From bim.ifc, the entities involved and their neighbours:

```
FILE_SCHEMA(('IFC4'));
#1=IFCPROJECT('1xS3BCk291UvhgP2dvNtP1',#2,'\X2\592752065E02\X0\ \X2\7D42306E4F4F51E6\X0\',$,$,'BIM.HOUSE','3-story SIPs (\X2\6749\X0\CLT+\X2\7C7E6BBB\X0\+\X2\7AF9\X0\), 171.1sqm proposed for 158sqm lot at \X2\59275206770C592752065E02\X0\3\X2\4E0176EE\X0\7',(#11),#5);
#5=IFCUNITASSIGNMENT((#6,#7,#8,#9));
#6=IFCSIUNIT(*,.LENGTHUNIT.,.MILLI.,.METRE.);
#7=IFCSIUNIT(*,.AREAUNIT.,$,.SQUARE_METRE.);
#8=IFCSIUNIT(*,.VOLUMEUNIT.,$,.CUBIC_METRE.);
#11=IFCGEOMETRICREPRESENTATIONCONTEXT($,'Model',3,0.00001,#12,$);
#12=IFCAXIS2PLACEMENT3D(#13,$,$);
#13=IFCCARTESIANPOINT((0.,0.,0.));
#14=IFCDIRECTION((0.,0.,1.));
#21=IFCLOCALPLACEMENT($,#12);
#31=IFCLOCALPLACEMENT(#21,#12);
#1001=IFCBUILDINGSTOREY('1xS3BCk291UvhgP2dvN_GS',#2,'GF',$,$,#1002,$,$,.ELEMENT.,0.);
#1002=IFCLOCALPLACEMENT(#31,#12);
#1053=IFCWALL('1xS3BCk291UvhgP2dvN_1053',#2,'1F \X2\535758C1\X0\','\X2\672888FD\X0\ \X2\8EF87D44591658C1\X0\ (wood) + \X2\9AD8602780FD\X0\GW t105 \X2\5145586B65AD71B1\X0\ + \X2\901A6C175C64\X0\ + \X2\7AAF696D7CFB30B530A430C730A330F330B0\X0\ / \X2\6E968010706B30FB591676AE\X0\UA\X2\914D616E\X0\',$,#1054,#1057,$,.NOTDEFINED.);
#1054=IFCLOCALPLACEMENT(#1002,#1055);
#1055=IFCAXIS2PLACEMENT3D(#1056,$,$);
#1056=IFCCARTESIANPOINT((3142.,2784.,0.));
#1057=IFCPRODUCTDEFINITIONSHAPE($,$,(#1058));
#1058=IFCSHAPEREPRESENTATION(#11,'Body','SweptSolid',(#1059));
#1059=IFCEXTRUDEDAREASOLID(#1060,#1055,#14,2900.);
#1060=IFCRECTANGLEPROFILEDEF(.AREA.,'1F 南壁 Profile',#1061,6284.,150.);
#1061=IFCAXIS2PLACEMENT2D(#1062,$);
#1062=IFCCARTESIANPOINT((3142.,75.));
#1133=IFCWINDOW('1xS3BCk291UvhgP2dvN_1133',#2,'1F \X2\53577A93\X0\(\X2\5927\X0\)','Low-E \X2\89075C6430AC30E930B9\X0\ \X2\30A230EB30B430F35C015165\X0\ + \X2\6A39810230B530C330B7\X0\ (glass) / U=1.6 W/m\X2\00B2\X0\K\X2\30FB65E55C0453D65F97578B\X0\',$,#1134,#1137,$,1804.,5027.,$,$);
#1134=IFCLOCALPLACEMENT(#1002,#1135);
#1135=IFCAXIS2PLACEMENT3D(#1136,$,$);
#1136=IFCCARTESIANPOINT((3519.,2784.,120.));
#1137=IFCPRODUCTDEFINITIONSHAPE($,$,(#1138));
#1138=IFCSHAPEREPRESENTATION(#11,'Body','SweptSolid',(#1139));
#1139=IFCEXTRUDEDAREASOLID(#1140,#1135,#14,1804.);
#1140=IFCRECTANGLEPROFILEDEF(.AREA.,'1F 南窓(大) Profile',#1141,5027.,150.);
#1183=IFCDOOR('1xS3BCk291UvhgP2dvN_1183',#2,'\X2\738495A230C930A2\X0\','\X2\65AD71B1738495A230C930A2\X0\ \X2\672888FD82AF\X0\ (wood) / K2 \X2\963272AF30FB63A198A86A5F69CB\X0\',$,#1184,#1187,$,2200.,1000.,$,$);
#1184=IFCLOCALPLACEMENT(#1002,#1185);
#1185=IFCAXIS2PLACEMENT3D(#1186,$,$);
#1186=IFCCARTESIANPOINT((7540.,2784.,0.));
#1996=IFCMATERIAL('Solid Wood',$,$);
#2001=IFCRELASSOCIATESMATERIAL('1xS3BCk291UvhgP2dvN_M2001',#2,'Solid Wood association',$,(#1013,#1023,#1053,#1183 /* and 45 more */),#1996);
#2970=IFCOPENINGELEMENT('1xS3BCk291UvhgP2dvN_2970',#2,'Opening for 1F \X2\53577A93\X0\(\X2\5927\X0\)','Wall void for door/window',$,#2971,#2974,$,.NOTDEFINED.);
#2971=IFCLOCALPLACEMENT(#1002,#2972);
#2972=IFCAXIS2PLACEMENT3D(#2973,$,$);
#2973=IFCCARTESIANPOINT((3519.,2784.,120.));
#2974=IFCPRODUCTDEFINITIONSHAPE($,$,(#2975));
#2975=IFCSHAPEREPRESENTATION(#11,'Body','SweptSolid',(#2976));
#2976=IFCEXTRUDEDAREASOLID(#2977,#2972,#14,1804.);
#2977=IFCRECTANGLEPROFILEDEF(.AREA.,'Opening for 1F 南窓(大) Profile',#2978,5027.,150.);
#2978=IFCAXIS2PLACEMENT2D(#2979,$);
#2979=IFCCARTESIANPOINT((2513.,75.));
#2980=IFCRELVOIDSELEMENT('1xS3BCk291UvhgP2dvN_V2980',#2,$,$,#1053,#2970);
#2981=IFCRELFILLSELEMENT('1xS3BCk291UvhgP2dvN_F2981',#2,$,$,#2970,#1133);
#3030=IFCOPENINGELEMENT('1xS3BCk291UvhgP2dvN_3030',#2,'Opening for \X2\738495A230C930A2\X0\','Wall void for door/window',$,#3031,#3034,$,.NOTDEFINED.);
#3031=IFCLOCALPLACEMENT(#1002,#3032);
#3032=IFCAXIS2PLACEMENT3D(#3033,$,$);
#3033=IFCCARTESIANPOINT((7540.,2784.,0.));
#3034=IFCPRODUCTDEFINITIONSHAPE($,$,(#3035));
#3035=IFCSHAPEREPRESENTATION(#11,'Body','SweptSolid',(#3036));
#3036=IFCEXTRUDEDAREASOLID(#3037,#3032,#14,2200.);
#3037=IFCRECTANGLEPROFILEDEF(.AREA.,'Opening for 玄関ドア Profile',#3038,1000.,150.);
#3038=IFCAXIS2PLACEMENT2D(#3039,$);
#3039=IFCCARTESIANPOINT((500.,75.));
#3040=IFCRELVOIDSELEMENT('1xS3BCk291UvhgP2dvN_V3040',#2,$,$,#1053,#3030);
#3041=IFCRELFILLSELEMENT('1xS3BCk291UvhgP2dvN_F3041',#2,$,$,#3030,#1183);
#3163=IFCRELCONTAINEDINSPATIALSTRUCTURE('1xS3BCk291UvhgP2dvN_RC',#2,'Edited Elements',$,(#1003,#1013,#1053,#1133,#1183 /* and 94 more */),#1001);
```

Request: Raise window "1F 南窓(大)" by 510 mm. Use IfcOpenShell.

```python
import numpy as np
import ifcopenshell
import ifcopenshell.api.geometry
import ifcopenshell.util.placement
import ifcopenshell.util.unit

model = ifcopenshell.open("bim.ifc")
unit_scale = ifcopenshell.util.unit.calculate_unit_scale(model)

window = model.by_id(1133)
opening = window.FillsVoids[0].RelatingOpeningElement
dz = 510.0

shift = np.array([0.0, 0.0, dz])
# The window is not placed relative to its opening, so move both.
for product in (opening, window):
    matrix = ifcopenshell.util.placement.get_local_placement(product.ObjectPlacement)
    matrix[:3, 3] += shift
    ifcopenshell.api.geometry.edit_object_placement(model, product=product, matrix=matrix, is_si=False)

print(f"moved by {dz * unit_scale:+.3f} m")

model.write("bim_edited.ifc")
```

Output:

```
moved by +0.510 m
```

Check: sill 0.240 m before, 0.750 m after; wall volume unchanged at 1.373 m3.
